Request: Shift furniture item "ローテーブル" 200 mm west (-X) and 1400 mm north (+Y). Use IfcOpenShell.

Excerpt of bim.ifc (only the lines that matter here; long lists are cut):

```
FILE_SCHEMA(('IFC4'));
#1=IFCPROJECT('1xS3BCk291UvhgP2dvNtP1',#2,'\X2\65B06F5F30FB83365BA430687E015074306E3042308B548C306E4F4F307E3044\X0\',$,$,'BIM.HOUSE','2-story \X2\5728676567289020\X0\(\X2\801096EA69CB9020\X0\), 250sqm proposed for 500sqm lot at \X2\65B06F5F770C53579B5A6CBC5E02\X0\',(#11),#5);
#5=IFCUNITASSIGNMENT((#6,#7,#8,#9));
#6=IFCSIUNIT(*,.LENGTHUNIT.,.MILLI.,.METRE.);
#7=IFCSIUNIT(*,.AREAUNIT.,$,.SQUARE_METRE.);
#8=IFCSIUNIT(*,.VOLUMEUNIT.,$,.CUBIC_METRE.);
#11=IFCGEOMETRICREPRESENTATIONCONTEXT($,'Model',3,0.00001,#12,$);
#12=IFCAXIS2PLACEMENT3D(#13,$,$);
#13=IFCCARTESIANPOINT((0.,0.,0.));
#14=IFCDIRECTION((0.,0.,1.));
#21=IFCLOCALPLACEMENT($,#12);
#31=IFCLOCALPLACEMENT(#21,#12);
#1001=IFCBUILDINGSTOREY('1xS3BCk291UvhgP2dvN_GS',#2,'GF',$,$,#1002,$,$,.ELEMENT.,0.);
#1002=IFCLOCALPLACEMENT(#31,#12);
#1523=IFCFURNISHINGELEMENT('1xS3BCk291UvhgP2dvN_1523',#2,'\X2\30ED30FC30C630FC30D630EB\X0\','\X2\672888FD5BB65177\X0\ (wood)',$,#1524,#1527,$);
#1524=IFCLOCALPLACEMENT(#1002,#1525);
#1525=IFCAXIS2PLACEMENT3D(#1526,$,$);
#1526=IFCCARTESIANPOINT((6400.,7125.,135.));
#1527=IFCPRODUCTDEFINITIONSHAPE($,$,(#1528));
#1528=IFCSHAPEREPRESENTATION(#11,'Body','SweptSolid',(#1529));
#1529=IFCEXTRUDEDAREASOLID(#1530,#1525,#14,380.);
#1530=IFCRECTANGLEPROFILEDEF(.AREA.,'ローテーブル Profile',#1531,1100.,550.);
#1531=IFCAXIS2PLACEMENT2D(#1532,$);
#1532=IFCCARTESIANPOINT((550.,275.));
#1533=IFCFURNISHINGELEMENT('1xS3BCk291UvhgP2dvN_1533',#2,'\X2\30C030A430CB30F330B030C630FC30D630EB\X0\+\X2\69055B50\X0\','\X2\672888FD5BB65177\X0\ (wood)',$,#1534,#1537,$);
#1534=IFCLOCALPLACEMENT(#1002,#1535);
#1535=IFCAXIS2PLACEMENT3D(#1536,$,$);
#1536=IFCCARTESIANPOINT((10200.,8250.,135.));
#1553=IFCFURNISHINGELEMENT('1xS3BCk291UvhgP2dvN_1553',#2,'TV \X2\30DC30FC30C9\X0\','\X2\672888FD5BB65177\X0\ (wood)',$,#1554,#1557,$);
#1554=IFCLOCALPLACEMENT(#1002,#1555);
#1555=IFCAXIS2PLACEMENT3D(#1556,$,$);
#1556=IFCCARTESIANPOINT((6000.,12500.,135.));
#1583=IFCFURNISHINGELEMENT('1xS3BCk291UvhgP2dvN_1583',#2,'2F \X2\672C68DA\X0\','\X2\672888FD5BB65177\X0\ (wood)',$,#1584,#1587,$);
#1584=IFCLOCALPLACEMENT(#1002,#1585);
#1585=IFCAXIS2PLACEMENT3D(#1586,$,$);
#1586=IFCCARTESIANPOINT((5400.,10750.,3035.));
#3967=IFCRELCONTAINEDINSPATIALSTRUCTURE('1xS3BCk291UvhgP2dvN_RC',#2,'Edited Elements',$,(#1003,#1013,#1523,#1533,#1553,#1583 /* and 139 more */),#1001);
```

```python
import ifcopenshell
import ifcopenshell.api.geometry
import ifcopenshell.util.placement
import ifcopenshell.util.unit

model = ifcopenshell.open("bim.ifc")
unit_scale = ifcopenshell.util.unit.calculate_unit_scale(model)

item = model.by_id(1523)
matrix = ifcopenshell.util.placement.get_local_placement(item.ObjectPlacement)
matrix[0, 3] -= 0.2 / unit_scale
matrix[1, 3] += 1.4 / unit_scale
ifcopenshell.api.geometry.edit_object_placement(model, product=item, matrix=matrix, is_si=False)

print(ifcopenshell.util.placement.get_local_placement(item.ObjectPlacement).round(3) + 0.0)

model.write("bim_rev.ifc")
```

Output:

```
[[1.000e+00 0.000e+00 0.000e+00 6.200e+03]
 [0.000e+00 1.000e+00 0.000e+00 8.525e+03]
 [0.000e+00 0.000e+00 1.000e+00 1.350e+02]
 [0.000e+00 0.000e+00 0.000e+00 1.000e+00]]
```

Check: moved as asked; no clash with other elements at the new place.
